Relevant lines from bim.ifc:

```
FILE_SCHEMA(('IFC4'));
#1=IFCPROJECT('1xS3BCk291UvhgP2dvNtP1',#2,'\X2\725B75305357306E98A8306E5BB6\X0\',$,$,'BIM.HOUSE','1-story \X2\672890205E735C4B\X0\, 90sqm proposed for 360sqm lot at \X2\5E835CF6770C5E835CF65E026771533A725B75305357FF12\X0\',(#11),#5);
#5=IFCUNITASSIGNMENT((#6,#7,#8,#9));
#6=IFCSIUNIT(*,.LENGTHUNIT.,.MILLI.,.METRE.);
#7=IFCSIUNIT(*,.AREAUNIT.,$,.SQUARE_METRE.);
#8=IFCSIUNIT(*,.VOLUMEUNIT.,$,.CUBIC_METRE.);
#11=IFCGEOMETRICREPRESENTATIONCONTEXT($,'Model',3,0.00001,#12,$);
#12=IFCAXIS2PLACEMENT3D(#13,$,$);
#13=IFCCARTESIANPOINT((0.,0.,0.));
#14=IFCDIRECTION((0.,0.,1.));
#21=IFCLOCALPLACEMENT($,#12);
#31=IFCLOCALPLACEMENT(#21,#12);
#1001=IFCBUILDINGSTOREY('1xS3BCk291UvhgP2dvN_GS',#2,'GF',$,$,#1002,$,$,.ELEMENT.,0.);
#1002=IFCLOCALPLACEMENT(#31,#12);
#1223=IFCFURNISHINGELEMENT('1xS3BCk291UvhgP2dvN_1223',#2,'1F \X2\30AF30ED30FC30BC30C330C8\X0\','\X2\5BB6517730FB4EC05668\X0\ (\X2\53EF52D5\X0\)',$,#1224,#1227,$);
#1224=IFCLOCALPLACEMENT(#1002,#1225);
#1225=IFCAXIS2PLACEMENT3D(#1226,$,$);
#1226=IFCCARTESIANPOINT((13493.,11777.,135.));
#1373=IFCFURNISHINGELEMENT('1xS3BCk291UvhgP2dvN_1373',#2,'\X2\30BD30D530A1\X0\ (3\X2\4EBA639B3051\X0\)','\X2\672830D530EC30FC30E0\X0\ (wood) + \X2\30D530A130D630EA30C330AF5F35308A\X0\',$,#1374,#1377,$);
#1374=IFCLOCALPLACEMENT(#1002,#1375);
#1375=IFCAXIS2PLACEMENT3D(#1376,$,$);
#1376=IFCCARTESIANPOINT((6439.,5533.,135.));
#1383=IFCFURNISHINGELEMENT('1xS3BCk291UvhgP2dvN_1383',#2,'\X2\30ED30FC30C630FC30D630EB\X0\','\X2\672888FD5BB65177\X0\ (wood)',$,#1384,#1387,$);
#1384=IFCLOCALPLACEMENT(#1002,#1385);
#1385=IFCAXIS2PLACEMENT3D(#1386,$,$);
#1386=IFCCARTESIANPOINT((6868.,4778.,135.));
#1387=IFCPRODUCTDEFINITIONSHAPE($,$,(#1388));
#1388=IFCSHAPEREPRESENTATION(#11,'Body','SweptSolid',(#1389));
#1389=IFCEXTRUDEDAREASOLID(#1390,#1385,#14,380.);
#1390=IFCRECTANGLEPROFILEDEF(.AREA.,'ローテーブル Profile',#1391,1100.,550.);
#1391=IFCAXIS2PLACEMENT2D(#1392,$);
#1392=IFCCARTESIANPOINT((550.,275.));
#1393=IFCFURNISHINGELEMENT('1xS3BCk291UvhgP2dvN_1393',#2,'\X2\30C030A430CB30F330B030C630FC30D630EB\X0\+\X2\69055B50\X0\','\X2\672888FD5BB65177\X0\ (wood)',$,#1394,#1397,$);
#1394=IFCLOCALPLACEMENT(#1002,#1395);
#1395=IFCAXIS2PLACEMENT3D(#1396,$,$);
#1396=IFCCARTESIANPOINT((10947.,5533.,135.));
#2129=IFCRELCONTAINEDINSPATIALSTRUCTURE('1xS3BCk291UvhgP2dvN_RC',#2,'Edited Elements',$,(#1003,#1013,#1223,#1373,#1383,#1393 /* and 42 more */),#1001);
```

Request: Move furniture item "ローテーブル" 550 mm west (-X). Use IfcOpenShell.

```python
import ifcopenshell
import ifcopenshell.api.geometry
import ifcopenshell.util.placement
import ifcopenshell.util.unit

model = ifcopenshell.open("bim.ifc")
unit_scale = ifcopenshell.util.unit.calculate_unit_scale(model)

item = model.by_guid("1xS3BCk291UvhgP2dvN_1383")
matrix = ifcopenshell.util.placement.get_local_placement(item.ObjectPlacement)
matrix[0, 3] -= 0.55 / unit_scale
ifcopenshell.api.geometry.edit_object_placement(model, product=item, matrix=matrix, is_si=False)

print(ifcopenshell.util.placement.get_local_placement(item.ObjectPlacement).round(3) + 0.0)

model.write("bim_v2.ifc")
```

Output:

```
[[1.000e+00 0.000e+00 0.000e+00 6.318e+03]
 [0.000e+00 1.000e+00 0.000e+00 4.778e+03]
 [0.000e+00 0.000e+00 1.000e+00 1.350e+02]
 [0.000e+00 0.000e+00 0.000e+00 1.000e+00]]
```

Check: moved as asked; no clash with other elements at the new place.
